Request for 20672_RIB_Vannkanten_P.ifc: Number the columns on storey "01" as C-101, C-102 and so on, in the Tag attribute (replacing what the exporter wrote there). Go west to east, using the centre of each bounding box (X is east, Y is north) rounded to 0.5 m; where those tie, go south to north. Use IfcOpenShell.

First a look at what the model holds.

```python
import ifcopenshell
import ifcopenshell.util.element
import ifcopenshell.util.placement

model = ifcopenshell.open("20672_RIB_Vannkanten_P.ifc")
print(model.schema)
storey = next(s for s in model.by_type("IfcBuildingStorey") if s.Name == "01")
columns = [e for e in ifcopenshell.util.element.get_decomposition(storey) if e.is_a("IfcColumn")]
for e in sorted(columns, key=lambda e: e.id()):
    origin = ifcopenshell.util.placement.get_local_placement(e.ObjectPlacement)[:3, 3]
    print(e.id(), e.Tag, e.Name, origin.round(2) + 0.0, sep=" | ")
```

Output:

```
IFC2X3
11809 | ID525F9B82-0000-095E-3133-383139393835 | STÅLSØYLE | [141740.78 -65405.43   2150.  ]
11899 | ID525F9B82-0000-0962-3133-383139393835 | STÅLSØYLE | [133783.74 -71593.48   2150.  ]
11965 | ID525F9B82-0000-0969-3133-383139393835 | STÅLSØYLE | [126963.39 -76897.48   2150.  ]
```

```python
import ifcopenshell
import ifcopenshell.geom
import ifcopenshell.util.element
import ifcopenshell.util.shape

model = ifcopenshell.open("20672_RIB_Vannkanten_P.ifc")
settings = ifcopenshell.geom.settings()
settings.set("use-world-coords", True)


def centre(element):
    shape = ifcopenshell.geom.create_shape(settings, element)
    return ifcopenshell.util.shape.get_bbox_centroid(shape.geometry)


storey = next(s for s in model.by_type("IfcBuildingStorey") if s.Name == "01")
columns = [e for e in ifcopenshell.util.element.get_decomposition(storey) if e.is_a("IfcColumn")]

# Insertion points can sit at a corner or the storey origin, so sort by the geometry (in metres).
centres = {e: centre(e) for e in columns}
columns.sort(key=lambda e: (round(centres[e][0] / 0.5), centres[e][1]))

for i, e in enumerate(columns, start=1):
    number = f"C-1{i:02d}"
    e.Tag = number
    print(e.id(), number)

model.write("20672_RIB_Vannkanten_P_v2.ifc")
```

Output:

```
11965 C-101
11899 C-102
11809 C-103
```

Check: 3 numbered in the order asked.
